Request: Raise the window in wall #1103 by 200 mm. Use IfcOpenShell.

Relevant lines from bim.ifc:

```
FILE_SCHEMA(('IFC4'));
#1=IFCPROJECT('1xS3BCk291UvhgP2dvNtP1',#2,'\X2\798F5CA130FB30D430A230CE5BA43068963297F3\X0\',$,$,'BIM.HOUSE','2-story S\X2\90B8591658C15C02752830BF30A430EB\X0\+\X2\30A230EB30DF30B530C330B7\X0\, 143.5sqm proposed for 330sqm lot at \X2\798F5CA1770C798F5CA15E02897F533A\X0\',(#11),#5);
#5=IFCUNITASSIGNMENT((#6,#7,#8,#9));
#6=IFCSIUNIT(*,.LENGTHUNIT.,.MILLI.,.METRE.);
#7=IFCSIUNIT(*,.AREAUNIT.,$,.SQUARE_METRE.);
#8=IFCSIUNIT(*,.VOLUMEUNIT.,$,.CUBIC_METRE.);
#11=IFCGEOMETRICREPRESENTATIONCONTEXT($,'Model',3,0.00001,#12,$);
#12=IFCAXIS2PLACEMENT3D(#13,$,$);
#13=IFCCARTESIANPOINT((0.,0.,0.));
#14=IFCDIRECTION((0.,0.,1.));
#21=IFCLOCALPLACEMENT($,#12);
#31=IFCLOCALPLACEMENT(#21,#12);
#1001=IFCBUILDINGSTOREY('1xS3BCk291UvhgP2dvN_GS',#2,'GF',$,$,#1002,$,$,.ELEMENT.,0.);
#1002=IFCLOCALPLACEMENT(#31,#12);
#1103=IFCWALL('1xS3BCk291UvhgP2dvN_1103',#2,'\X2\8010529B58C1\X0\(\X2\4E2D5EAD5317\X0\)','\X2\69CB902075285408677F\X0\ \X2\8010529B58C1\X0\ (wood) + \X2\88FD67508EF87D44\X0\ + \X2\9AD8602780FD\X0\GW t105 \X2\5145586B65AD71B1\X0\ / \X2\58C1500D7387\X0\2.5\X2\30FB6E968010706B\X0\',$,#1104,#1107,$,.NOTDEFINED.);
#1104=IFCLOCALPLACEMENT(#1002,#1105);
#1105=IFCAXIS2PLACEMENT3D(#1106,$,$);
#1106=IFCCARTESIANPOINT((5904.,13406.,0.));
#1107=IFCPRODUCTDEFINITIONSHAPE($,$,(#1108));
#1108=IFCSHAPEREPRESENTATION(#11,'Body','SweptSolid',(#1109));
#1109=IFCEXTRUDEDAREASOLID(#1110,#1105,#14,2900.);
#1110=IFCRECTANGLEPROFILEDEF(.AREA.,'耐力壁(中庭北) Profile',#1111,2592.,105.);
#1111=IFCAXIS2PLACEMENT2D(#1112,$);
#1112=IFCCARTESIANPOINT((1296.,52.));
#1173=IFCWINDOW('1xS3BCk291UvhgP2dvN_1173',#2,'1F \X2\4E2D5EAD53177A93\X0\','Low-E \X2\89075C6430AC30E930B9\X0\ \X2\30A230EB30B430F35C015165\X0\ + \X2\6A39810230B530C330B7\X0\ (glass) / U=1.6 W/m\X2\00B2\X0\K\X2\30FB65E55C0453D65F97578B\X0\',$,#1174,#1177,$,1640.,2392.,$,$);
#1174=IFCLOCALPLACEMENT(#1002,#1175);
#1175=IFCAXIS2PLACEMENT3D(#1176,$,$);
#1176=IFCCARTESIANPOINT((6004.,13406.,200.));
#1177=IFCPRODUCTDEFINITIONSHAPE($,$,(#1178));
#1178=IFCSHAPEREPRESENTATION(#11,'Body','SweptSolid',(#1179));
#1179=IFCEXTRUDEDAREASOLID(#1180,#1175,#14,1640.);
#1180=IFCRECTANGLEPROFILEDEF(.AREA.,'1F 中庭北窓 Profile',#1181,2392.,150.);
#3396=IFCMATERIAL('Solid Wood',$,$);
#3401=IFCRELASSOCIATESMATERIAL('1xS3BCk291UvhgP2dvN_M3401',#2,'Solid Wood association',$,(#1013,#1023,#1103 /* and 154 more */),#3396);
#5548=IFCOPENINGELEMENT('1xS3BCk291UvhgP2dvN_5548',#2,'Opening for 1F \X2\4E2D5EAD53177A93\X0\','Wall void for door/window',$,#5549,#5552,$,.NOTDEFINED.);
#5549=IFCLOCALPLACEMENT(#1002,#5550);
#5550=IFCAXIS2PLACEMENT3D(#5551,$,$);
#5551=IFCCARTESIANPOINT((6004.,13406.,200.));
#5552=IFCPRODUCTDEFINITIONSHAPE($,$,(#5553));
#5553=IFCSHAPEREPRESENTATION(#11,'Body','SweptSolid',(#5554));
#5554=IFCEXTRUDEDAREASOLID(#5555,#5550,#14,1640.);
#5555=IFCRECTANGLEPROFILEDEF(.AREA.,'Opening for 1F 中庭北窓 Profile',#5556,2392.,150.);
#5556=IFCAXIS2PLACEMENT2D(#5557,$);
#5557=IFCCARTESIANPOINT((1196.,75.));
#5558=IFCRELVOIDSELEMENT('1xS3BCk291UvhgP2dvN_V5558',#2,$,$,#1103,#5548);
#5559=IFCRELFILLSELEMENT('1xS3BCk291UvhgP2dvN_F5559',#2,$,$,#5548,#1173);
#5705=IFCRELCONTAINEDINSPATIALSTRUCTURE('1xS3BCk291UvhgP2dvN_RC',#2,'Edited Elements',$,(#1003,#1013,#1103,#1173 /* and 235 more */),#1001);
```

```python
import numpy as np
import ifcopenshell
import ifcopenshell.api.geometry
import ifcopenshell.util.placement
import ifcopenshell.util.unit

model = ifcopenshell.open("bim.ifc")
unit_scale = ifcopenshell.util.unit.calculate_unit_scale(model)

window = model.by_guid("1xS3BCk291UvhgP2dvN_1173")
opening = window.FillsVoids[0].RelatingOpeningElement
dz = 200.0

shift = np.array([0.0, 0.0, dz])
# The window is not placed relative to its opening, so move both.
for product in (opening, window):
    matrix = ifcopenshell.util.placement.get_local_placement(product.ObjectPlacement)
    matrix[:3, 3] += shift
    ifcopenshell.api.geometry.edit_object_placement(model, product=product, matrix=matrix, is_si=False)

print(f"moved by {dz * unit_scale:+.3f} m")

model.write("bim_rev.ifc")
```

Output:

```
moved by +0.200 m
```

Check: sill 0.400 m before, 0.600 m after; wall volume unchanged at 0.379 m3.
